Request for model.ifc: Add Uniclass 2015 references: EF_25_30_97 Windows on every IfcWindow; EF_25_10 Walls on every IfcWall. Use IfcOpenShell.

First a look at what the model holds.

```python
import ifcopenshell

model = ifcopenshell.open("model.ifc")
print(model.schema)
print("classifications:", [c.Name for c in model.by_type("IfcClassification")])
for ifc_class in ("IfcDoor", "IfcRoof", "IfcStair", "IfcWall", "IfcWindow"):
    print(ifc_class, len(model.by_type(ifc_class)))
```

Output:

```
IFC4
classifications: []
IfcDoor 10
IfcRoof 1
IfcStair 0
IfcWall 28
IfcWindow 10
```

```python
import ifcopenshell
import ifcopenshell.api.classification

model = ifcopenshell.open("model.ifc")

system = ifcopenshell.api.classification.add_classification(model, classification="Uniclass 2015")

codes = {
    "IfcWindow": ("EF_25_30_97", "Windows"),
    "IfcWall": ("EF_25_10", "Walls"),
}
for ifc_class, (code, name) in codes.items():
    products = model.by_type(ifc_class)
    ifcopenshell.api.classification.add_reference(
        model, products=products, classification=system, identification=code, name=name
    )
    print(code, len(products))

model.write("model_v2.ifc")
```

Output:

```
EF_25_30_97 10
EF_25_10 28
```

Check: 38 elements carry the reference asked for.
